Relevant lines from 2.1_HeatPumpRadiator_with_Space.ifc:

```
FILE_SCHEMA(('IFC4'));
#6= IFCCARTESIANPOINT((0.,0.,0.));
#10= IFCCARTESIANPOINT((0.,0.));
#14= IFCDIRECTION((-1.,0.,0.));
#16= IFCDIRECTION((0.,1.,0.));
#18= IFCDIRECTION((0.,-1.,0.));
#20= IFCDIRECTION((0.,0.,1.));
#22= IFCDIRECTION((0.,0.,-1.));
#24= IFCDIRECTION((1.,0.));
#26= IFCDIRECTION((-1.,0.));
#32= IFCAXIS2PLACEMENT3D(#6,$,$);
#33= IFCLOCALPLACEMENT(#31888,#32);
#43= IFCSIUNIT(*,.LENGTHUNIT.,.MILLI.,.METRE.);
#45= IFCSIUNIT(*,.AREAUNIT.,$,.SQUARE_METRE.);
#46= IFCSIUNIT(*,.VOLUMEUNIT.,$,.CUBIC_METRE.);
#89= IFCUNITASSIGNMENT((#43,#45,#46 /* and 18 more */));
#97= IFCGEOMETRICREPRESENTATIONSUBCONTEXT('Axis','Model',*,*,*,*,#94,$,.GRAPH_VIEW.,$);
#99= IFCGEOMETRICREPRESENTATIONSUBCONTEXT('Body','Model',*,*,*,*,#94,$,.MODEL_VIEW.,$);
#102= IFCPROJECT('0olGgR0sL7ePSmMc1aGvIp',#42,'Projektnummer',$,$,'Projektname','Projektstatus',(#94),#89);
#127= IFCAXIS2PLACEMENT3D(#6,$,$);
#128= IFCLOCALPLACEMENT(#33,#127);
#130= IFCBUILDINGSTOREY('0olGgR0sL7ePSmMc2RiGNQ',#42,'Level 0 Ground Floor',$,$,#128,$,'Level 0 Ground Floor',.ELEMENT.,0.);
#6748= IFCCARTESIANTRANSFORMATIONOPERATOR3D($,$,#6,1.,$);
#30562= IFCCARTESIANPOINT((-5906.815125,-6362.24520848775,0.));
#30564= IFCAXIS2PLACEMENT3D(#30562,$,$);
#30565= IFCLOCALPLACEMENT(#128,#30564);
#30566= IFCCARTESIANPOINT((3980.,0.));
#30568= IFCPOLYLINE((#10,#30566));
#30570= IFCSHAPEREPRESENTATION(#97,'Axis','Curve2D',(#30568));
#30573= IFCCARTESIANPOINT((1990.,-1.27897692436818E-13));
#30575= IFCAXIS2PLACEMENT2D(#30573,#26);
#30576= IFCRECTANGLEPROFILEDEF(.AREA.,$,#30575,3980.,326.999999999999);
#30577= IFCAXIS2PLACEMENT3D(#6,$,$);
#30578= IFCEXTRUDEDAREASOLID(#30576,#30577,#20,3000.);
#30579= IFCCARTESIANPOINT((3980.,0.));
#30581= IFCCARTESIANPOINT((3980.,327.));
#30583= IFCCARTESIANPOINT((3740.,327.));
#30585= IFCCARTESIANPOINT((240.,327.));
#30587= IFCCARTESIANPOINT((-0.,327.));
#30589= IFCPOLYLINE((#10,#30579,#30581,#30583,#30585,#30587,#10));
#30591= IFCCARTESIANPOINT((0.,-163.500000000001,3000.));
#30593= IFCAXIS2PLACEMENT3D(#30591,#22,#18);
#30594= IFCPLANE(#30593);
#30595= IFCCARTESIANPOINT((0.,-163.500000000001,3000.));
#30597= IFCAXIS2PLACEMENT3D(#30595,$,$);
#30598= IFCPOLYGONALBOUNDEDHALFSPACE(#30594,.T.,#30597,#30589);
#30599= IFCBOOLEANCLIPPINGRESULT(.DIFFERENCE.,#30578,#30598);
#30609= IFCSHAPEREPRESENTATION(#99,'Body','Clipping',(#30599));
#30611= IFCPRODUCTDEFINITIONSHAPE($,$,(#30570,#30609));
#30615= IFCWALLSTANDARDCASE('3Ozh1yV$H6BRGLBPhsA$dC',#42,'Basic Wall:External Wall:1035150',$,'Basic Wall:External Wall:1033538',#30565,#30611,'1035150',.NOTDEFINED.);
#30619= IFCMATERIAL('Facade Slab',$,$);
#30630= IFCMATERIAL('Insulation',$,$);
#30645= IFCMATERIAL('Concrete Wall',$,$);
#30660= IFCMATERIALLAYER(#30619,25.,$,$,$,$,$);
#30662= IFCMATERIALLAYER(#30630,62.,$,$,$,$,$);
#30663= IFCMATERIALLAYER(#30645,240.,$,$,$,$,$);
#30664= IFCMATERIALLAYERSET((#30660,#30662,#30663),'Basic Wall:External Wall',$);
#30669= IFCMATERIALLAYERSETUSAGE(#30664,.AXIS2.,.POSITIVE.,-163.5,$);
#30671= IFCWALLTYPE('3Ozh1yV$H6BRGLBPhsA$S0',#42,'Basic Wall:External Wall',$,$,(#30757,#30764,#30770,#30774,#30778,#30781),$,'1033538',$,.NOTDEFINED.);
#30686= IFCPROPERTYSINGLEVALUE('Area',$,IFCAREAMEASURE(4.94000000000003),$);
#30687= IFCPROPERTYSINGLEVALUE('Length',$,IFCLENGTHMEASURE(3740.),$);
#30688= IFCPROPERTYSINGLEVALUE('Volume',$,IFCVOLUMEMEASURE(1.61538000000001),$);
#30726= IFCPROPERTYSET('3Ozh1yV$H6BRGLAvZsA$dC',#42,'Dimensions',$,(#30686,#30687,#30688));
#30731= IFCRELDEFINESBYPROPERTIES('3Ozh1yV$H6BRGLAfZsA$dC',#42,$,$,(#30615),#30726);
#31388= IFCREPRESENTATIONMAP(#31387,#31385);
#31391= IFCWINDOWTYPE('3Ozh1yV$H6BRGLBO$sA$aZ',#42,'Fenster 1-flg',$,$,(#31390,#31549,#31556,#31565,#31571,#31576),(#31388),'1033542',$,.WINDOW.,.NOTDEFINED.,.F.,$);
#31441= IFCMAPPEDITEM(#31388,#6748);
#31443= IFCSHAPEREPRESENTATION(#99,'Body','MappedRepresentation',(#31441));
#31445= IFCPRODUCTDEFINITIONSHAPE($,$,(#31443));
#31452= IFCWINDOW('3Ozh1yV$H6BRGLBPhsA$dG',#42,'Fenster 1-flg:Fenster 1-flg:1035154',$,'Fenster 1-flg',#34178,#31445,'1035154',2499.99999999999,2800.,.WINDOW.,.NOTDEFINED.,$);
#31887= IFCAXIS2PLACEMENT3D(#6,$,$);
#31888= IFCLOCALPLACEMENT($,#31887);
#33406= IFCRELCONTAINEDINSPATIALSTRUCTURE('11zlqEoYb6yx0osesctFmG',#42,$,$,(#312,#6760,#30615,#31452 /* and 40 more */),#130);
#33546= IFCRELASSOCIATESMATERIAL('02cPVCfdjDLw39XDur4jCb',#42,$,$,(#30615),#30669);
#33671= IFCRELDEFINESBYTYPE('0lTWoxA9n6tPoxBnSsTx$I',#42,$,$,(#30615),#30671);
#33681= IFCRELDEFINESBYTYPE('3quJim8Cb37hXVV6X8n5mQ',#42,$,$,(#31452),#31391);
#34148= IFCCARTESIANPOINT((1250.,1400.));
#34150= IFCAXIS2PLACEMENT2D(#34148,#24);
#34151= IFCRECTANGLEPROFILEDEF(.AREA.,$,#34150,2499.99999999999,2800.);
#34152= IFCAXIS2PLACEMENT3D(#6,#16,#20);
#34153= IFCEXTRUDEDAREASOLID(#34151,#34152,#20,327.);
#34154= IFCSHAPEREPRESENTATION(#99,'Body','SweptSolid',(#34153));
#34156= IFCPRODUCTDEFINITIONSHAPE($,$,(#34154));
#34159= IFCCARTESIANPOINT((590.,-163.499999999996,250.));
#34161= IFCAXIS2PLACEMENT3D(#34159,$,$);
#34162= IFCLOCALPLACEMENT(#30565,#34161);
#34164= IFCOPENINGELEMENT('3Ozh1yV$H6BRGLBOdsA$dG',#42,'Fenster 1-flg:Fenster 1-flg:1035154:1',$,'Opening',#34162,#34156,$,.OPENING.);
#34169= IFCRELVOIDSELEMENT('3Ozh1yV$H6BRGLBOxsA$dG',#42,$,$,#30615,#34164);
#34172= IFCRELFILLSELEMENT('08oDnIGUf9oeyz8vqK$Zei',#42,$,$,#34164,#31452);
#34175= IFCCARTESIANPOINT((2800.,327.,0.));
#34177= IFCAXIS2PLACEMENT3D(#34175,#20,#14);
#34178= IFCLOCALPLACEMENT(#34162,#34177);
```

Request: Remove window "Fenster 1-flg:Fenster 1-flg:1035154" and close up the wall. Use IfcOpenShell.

```python
import ifcopenshell
import ifcopenshell.api.feature
import ifcopenshell.api.pset
import ifcopenshell.api.root
import ifcopenshell.geom
import ifcopenshell.util.element
import ifcopenshell.util.shape
import ifcopenshell.util.unit

model = ifcopenshell.open("2.1_HeatPumpRadiator_with_Space.ifc")
area_scale = ifcopenshell.util.unit.calculate_unit_scale(model, "AREAUNIT")
volume_scale = ifcopenshell.util.unit.calculate_unit_scale(model, "VOLUMEUNIT")
settings = ifcopenshell.geom.settings()


def volume(element):
    """Net volume in cubic metres, openings subtracted."""
    shape = ifcopenshell.geom.create_shape(settings, element)
    return ifcopenshell.util.shape.get_volume(shape.geometry)


window = model.by_id(31452)
opening = window.FillsVoids[0].RelatingOpeningElement
wall = opening.VoidsElements[0].RelatingBuildingElement
before = volume(wall)

ifcopenshell.api.root.remove_product(model, product=window)
ifcopenshell.api.feature.remove_feature(model, feature=opening)

after = volume(wall)
thickness = 0.327  # wall thickness in metres

# Update the wall's stored quantities.
pset = model.by_id(ifcopenshell.util.element.get_pset(wall, "Dimensions", should_inherit=False)["id"])
ifcopenshell.api.pset.edit_pset(model, pset=pset, properties={
    "Area": model.create_entity("IfcAreaMeasure", after / thickness / area_scale),
    "Volume": model.create_entity("IfcVolumeMeasure", after / volume_scale),
})

print(f"wall volume {before:.3f} -> {after:.3f} m3")

model.write("2.1_HeatPumpRadiator_with_Space_rev.ifc")
```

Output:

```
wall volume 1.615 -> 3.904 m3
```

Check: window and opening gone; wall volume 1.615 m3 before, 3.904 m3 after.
